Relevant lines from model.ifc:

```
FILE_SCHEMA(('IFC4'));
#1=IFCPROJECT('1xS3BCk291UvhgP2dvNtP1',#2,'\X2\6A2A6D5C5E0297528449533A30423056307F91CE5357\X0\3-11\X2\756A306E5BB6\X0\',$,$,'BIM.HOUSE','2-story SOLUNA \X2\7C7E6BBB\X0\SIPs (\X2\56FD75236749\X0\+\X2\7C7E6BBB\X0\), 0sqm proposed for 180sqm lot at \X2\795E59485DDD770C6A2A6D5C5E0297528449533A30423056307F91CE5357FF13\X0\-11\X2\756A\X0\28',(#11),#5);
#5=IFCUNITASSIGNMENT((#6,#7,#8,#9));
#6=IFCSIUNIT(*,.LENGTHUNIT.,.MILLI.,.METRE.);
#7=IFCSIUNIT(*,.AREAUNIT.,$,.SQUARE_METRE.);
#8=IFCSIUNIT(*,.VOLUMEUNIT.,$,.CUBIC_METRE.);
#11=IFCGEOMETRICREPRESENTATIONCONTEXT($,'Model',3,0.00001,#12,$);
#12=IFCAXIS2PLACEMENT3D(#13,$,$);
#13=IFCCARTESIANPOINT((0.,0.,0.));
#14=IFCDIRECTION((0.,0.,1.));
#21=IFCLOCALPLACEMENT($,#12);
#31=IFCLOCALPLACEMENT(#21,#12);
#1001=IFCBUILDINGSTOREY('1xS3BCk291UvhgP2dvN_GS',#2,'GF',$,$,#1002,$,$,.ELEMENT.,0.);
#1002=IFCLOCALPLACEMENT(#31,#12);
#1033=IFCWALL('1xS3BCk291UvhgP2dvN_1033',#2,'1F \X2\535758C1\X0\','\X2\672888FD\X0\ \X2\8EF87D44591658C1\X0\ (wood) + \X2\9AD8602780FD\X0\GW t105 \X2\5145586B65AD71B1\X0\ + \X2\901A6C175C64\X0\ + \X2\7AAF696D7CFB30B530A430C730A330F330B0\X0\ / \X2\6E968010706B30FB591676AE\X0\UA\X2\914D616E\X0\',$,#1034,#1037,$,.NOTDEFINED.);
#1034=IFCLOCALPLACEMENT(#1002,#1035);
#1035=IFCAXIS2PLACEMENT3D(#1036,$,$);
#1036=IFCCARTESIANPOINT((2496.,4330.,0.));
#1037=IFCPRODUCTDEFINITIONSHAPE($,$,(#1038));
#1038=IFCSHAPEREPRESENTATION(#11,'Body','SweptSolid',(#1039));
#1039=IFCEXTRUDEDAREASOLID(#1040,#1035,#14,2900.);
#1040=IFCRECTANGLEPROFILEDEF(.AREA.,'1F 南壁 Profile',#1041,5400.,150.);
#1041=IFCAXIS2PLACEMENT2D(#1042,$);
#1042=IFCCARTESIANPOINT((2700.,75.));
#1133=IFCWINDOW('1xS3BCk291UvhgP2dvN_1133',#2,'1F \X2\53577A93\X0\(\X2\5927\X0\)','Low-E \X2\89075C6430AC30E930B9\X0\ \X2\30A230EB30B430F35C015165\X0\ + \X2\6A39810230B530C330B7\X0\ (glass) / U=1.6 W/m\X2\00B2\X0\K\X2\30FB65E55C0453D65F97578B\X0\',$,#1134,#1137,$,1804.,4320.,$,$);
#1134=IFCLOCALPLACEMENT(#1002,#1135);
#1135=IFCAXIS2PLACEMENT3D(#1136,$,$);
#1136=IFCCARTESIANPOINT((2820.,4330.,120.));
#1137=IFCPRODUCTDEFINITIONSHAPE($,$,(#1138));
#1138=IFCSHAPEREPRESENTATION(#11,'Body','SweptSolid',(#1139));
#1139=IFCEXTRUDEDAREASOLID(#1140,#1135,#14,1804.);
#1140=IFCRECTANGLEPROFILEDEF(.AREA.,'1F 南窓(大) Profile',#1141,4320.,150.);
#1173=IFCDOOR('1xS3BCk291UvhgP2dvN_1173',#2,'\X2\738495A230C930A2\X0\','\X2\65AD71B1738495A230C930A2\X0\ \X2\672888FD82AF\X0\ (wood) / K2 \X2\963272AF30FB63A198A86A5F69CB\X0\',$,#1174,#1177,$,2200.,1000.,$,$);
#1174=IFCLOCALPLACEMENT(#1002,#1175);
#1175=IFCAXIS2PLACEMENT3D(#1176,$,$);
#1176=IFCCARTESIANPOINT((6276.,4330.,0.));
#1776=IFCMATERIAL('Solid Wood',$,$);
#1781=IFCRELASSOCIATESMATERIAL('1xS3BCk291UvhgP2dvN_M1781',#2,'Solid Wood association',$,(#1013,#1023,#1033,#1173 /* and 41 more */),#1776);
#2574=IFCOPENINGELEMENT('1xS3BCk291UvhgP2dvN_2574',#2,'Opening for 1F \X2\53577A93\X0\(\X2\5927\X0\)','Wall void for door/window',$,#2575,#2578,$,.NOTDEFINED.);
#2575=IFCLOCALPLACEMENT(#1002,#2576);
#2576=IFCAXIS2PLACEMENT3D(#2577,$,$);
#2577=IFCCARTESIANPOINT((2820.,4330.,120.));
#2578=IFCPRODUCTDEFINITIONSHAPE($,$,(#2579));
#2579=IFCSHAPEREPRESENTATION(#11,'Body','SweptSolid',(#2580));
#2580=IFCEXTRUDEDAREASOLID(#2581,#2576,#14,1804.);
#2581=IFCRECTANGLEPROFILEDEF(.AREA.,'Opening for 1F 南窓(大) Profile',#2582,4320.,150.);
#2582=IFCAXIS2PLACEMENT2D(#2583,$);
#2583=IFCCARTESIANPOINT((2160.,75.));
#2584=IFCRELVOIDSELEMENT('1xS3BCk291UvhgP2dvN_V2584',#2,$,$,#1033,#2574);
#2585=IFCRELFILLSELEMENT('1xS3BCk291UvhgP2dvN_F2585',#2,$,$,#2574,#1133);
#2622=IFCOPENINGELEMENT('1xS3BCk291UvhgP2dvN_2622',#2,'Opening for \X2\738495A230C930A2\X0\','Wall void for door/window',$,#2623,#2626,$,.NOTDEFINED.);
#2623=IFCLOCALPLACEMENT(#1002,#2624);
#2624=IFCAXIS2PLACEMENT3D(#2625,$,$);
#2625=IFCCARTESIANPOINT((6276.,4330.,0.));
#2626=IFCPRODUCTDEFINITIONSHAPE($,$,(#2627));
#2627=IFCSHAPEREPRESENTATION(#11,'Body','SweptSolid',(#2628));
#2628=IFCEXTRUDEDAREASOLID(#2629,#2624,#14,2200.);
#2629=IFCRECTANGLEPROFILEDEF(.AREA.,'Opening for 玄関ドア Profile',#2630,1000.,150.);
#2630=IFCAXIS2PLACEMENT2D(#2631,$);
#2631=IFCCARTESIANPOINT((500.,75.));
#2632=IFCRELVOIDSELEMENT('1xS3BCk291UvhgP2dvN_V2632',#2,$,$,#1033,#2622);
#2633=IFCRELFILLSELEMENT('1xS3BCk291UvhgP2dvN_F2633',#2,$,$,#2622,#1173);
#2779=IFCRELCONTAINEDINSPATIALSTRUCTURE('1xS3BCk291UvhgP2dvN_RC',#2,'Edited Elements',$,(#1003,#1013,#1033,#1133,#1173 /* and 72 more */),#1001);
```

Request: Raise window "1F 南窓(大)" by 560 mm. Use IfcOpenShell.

```python
import numpy as np
import ifcopenshell
import ifcopenshell.api.geometry
import ifcopenshell.util.placement
import ifcopenshell.util.unit

model = ifcopenshell.open("model.ifc")
unit_scale = ifcopenshell.util.unit.calculate_unit_scale(model)

window = model.by_guid("1xS3BCk291UvhgP2dvN_1133")
opening = window.FillsVoids[0].RelatingOpeningElement
dz = 560.0

shift = np.array([0.0, 0.0, dz])
# The window is not placed relative to its opening, so move both.
for product in (opening, window):
    matrix = ifcopenshell.util.placement.get_local_placement(product.ObjectPlacement)
    matrix[:3, 3] += shift
    ifcopenshell.api.geometry.edit_object_placement(model, product=product, matrix=matrix, is_si=False)

print(f"moved by {dz * unit_scale:+.3f} m")

model.write("model_updated.ifc")
```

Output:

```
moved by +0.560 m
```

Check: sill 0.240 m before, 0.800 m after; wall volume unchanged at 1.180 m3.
